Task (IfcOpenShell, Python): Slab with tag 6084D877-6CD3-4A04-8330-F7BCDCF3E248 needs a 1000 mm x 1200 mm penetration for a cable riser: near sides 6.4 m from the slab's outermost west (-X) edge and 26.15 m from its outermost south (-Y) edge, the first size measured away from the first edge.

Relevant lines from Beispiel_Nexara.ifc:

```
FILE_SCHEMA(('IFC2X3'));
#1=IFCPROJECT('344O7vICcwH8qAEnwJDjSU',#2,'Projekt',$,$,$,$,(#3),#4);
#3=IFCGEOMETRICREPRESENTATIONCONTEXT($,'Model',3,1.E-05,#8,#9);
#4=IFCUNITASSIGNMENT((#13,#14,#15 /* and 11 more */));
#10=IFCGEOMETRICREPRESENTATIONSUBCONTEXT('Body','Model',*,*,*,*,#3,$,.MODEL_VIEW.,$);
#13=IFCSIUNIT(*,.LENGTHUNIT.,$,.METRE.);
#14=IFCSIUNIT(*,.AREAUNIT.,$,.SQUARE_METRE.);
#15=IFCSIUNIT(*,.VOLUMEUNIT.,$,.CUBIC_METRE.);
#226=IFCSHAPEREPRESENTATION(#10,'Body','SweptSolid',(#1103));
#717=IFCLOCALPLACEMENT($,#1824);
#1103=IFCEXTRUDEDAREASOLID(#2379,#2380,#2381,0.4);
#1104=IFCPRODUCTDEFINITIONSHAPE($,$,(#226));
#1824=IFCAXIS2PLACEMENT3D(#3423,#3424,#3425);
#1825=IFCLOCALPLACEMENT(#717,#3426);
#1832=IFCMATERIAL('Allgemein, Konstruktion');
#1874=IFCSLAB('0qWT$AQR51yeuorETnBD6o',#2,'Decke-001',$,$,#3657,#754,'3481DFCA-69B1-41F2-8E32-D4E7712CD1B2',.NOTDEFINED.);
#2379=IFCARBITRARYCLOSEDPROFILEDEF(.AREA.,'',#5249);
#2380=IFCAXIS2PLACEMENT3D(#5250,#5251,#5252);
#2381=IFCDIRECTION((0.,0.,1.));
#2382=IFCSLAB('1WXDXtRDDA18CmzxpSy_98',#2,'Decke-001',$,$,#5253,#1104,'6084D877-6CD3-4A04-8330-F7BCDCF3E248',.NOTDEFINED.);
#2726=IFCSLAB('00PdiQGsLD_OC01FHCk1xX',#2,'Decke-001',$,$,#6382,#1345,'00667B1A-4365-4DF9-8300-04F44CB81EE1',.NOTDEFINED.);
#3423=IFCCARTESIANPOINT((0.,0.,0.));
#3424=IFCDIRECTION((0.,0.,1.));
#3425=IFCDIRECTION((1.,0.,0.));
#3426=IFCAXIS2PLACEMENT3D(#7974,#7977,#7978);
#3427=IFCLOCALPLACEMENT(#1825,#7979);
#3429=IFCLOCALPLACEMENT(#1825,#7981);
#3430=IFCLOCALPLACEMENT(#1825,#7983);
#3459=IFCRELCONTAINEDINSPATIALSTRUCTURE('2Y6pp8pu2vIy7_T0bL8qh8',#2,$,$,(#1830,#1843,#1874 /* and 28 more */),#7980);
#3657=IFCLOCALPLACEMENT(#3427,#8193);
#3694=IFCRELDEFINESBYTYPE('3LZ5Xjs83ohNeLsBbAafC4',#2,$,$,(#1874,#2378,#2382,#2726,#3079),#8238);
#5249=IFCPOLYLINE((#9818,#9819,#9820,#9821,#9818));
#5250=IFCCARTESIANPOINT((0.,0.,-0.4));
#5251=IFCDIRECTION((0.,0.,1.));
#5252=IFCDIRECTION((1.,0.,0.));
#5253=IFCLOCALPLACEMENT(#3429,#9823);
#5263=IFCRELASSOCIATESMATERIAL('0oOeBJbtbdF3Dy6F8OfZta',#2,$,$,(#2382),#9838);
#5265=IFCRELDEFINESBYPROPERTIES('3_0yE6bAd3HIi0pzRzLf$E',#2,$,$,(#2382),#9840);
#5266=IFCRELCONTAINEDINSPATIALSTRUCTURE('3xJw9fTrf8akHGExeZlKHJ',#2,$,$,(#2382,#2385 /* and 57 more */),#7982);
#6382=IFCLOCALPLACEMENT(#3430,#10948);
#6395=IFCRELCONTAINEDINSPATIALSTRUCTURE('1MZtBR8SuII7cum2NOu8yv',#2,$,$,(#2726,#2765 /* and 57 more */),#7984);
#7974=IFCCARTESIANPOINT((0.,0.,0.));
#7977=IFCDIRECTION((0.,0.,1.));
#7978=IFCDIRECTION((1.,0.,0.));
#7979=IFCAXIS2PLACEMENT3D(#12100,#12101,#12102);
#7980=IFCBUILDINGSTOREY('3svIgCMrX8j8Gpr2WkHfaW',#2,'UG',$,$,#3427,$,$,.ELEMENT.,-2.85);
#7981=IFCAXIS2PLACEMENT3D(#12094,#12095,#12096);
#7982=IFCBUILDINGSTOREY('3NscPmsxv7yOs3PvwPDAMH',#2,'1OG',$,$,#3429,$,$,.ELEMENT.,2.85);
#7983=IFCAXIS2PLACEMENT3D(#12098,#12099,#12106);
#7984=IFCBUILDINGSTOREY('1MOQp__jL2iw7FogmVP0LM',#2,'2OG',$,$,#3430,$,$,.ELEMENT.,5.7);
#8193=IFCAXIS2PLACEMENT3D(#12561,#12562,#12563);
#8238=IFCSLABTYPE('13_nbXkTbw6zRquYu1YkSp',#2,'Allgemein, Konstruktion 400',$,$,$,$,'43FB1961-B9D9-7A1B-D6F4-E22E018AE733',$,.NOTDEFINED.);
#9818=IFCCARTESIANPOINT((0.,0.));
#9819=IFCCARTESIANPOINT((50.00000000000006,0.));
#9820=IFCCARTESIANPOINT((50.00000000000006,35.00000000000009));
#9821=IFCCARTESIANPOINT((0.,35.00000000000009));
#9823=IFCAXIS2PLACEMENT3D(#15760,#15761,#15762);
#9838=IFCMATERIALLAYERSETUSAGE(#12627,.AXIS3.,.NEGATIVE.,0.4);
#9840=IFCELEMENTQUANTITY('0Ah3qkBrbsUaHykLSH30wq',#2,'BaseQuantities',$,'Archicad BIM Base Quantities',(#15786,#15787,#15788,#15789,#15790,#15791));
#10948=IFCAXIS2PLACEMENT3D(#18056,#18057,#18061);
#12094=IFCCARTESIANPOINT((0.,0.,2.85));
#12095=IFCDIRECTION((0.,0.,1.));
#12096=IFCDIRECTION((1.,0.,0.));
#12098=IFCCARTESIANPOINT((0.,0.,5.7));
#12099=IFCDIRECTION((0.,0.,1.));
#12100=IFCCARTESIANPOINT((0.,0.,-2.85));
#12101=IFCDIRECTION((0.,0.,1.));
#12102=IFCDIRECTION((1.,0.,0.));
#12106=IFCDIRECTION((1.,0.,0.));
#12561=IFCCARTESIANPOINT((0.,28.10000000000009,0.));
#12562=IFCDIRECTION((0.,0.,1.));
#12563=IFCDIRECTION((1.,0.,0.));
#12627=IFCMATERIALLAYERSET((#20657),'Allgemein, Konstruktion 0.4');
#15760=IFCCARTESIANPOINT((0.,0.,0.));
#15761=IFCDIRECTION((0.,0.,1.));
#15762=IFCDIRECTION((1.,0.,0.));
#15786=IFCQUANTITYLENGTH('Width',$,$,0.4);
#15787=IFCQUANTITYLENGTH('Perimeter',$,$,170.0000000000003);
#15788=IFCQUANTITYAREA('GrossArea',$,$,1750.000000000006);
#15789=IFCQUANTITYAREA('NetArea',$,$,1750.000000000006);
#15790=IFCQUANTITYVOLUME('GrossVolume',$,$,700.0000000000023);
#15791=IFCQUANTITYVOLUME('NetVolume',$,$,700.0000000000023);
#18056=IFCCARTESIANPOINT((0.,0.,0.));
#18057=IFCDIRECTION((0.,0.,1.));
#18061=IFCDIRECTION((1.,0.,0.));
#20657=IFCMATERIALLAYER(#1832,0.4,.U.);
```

```python
import numpy as np
import ifcopenshell
import ifcopenshell.api.feature
import ifcopenshell.api.geometry
import ifcopenshell.api.pset
import ifcopenshell.api.root
import ifcopenshell.geom
import ifcopenshell.util.element
import ifcopenshell.util.placement
import ifcopenshell.util.representation
import ifcopenshell.util.shape
import ifcopenshell.util.unit

model = ifcopenshell.open("Beispiel_Nexara.ifc")
unit_scale = ifcopenshell.util.unit.calculate_unit_scale(model)
area_scale = ifcopenshell.util.unit.calculate_unit_scale(model, "AREAUNIT")
volume_scale = ifcopenshell.util.unit.calculate_unit_scale(model, "VOLUMEUNIT")
settings = ifcopenshell.geom.settings()


def volume(element):
    """Net volume in cubic metres, openings subtracted."""
    shape = ifcopenshell.geom.create_shape(settings, element)
    return ifcopenshell.util.shape.get_volume(shape.geometry)


slab = model.by_guid("1WXDXtRDDA18CmzxpSy_98")
before = volume(slab)

# Extent in the slab's own axes, in metres. The edges named are its -X and -Y sides.
slab_shape = ifcopenshell.geom.create_shape(settings, slab)
vertices = ifcopenshell.util.shape.get_vertices(slab_shape.geometry)
x_min, y_min, bottom = vertices.min(axis=0)
top = vertices[:, 2].max()

opening = ifcopenshell.api.root.create_entity(model, ifc_class="IfcOpeningElement", name="Cable riser opening")
context = ifcopenshell.util.representation.get_context(model, "Model", "Body", "MODEL_VIEW")
width, depth = 1, 1.2
outline = [(0.0, 0.0), (width, 0.0), (width, depth), (0.0, depth), (0.0, 0.0)]
# Overshoot both faces by 50 mm so the cut is clean.
shape = ifcopenshell.api.geometry.add_slab_representation(
    model, context=context, depth=top - bottom + 0.1, polyline=outline
)
ifcopenshell.api.geometry.assign_representation(model, product=opening, representation=shape)

matrix = ifcopenshell.util.placement.get_local_placement(slab.ObjectPlacement)
matrix[:, 3] = matrix @ np.append(np.array([x_min + 6.4, y_min + 26.15, bottom - 0.05]) / unit_scale, 1.0)
ifcopenshell.api.geometry.edit_object_placement(model, product=opening, matrix=matrix, is_si=False)
ifcopenshell.api.feature.add_feature(model, feature=opening, element=slab)

after = volume(slab)

# Update the slab's stored quantities.
qto = model.by_id(ifcopenshell.util.element.get_pset(slab, "BaseQuantities", should_inherit=False)["id"])
ifcopenshell.api.pset.edit_qto(model, qto=qto, properties={
    "NetArea": after / (top - bottom) / area_scale,
    "NetVolume": after / volume_scale,
})

print(f"slab volume {before:.3f} -> {after:.3f} m3")

model.write("Beispiel_Nexara_v2.ifc")
```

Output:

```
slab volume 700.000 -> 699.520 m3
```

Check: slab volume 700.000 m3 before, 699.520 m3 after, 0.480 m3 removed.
